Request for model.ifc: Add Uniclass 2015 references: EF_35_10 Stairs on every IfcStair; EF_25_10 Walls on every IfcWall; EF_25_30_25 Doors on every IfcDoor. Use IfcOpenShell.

First a look at what the model holds.

```python
import ifcopenshell

model = ifcopenshell.open("model.ifc")
print(model.schema)
print("classifications:", [c.Name for c in model.by_type("IfcClassification")])
for ifc_class in ("IfcDoor", "IfcRoof", "IfcStair", "IfcWall", "IfcWindow"):
    print(ifc_class, len(model.by_type(ifc_class)))
```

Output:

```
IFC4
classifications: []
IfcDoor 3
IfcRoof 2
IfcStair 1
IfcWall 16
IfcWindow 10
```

```python
import ifcopenshell
import ifcopenshell.api.classification

model = ifcopenshell.open("model.ifc")

system = ifcopenshell.api.classification.add_classification(model, classification="Uniclass 2015")

codes = {
    "IfcStair": ("EF_35_10", "Stairs"),
    "IfcWall": ("EF_25_10", "Walls"),
    "IfcDoor": ("EF_25_30_25", "Doors"),
}
for ifc_class, (code, name) in codes.items():
    products = model.by_type(ifc_class)
    ifcopenshell.api.classification.add_reference(
        model, products=products, classification=system, identification=code, name=name
    )
    print(code, len(products))

model.write("model-out.ifc")
```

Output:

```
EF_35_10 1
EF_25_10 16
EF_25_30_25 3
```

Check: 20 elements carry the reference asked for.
